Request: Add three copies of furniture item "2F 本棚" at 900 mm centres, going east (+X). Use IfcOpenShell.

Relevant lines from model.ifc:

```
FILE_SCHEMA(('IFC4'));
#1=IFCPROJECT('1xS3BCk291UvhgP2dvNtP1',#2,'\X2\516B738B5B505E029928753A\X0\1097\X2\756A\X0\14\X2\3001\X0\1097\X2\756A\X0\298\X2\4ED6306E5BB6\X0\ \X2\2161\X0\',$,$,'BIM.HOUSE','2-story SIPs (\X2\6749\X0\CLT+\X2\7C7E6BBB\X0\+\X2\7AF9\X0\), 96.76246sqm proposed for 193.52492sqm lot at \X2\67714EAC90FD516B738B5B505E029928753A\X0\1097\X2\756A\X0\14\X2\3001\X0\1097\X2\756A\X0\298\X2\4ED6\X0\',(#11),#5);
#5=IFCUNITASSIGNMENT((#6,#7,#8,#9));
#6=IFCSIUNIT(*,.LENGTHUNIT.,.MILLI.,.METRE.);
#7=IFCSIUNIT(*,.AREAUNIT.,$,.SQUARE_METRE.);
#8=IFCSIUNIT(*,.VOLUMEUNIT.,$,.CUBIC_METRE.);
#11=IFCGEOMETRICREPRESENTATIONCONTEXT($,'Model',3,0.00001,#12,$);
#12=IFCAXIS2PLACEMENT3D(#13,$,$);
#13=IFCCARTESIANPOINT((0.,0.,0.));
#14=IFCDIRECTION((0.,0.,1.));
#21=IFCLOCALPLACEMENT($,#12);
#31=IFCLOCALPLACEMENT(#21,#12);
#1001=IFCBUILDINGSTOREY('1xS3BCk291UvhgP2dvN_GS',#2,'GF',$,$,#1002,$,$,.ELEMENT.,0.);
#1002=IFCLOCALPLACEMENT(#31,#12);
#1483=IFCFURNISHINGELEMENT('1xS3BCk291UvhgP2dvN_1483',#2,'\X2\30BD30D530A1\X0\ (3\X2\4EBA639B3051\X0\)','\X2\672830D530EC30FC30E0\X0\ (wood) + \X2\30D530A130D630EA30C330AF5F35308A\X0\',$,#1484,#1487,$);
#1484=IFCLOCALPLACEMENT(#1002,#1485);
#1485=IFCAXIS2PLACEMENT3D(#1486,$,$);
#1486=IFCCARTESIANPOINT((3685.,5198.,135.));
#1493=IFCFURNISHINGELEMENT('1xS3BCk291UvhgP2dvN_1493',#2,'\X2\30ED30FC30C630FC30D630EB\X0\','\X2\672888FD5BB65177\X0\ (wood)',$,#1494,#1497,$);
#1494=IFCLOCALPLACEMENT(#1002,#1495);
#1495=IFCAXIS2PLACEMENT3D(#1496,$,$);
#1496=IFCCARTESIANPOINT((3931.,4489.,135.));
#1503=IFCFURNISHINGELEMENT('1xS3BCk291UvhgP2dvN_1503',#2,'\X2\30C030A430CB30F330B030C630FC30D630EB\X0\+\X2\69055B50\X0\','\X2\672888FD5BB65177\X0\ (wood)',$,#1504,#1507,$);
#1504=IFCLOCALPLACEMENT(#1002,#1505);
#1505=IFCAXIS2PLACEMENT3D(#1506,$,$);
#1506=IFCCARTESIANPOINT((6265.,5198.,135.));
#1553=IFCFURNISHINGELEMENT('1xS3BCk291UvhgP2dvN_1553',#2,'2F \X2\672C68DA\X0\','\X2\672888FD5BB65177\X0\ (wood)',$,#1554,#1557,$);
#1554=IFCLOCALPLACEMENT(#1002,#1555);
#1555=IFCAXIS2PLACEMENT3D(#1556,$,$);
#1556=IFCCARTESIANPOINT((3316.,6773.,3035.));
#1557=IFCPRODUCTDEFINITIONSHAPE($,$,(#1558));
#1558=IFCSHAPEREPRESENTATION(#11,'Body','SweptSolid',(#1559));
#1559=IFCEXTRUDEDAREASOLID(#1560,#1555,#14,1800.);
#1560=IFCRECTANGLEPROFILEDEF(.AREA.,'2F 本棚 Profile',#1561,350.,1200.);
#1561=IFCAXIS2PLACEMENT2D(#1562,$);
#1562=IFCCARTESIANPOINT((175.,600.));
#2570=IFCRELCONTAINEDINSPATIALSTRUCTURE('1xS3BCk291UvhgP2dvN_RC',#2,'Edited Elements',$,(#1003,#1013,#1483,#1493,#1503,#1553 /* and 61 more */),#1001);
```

```python
import numpy as np
import ifcopenshell
import ifcopenshell.api.geometry
import ifcopenshell.api.root
import ifcopenshell.util.element
import ifcopenshell.util.placement
import ifcopenshell.util.unit

model = ifcopenshell.open("model.ifc")
unit_scale = ifcopenshell.util.unit.calculate_unit_scale(model)


def reuse_history(source, copy):
    """copy_class also copies each property set's owner history, people and application; keep the originals."""
    for rel in copy.IsDefinedBy:
        if rel.is_a("IfcRelDefinesByProperties") and (history := rel.RelatingPropertyDefinition.OwnerHistory):
            rel.RelatingPropertyDefinition.OwnerHistory = source.OwnerHistory
            ifcopenshell.util.element.remove_deep2(model, history)


source = model.by_id(1553)
base = ifcopenshell.util.placement.get_local_placement(source.ObjectPlacement)
step = np.array([1.0, 0.0, 0.0]) * 0.9 / unit_scale

for i in range(1, 4):
    copy = ifcopenshell.api.root.copy_class(model, product=source)
    copy.Representation = ifcopenshell.util.element.copy_deep(
        model, source.Representation, exclude=["IfcGeometricRepresentationContext", "IfcRepresentationMap"]
    )
    reuse_history(source, copy)
    matrix = base.copy()
    matrix[:3, 3] += i * step
    print("added at", matrix[:3, 3].round(3) + 0.0)
    ifcopenshell.api.geometry.edit_object_placement(model, product=copy, matrix=matrix, is_si=False)

model.write("model_v2.ifc")
```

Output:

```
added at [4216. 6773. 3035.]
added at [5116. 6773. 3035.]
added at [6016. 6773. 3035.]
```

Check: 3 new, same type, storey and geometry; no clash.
